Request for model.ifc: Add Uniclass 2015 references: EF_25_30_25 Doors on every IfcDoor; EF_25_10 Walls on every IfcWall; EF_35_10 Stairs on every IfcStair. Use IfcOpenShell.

First a look at what the model holds.

```python
import ifcopenshell

model = ifcopenshell.open("model.ifc")
print(model.schema)
print("classifications:", [c.Name for c in model.by_type("IfcClassification")])
for ifc_class in ("IfcDoor", "IfcRoof", "IfcStair", "IfcWall", "IfcWindow"):
    print(ifc_class, len(model.by_type(ifc_class)))
```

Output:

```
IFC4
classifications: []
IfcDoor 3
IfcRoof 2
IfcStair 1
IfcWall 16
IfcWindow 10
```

```python
import ifcopenshell
import ifcopenshell.api.classification

model = ifcopenshell.open("model.ifc")

system = ifcopenshell.api.classification.add_classification(model, classification="Uniclass 2015")

codes = {
    "IfcDoor": ("EF_25_30_25", "Doors"),
    "IfcWall": ("EF_25_10", "Walls"),
    "IfcStair": ("EF_35_10", "Stairs"),
}
for ifc_class, (code, name) in codes.items():
    products = model.by_type(ifc_class)
    ifcopenshell.api.classification.add_reference(
        model, products=products, classification=system, identification=code, name=name
    )
    print(code, len(products))

model.write("model-out.ifc")
```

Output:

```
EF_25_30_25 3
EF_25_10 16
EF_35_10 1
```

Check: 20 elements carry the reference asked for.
